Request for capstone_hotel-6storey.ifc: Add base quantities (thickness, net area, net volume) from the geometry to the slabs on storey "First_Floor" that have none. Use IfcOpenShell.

First a look at what the model holds.

```python
import ifcopenshell
import ifcopenshell.util.element
import ifcopenshell.util.unit

model = ifcopenshell.open("capstone_hotel-6storey.ifc")
print(model.schema)
for unit_type in ("LENGTHUNIT", "AREAUNIT", "VOLUMEUNIT"):
    print(unit_type, ifcopenshell.util.unit.calculate_unit_scale(model, unit_type))
storey = next(s for s in model.by_type("IfcBuildingStorey") if s.Name == "First_Floor")
slabs = [e for e in ifcopenshell.util.element.get_decomposition(storey) if e.is_a("IfcSlab")]
for e in sorted(slabs, key=lambda e: e.id()):
    print(e.id(), e.is_a(), e.Name, list(ifcopenshell.util.element.get_psets(e, qtos_only=True)), sep=" | ")
```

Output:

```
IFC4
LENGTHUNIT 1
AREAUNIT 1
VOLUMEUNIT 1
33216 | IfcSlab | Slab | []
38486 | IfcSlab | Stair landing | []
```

```python
import ifcopenshell
import ifcopenshell.api.pset
import ifcopenshell.geom
import ifcopenshell.util.element
import ifcopenshell.util.shape
import ifcopenshell.util.unit

model = ifcopenshell.open("capstone_hotel-6storey.ifc")
unit_scale = ifcopenshell.util.unit.calculate_unit_scale(model)
area_scale = ifcopenshell.util.unit.calculate_unit_scale(model, "AREAUNIT")
volume_scale = ifcopenshell.util.unit.calculate_unit_scale(model, "VOLUMEUNIT")
settings = ifcopenshell.geom.settings()

storey = next(s for s in model.by_type("IfcBuildingStorey") if s.Name == "First_Floor")
slabs = [e for e in ifcopenshell.util.element.get_decomposition(storey) if e.is_a("IfcSlab")]

for e in sorted(slabs, key=lambda e: e.id()):
    if ifcopenshell.util.element.get_psets(e, qtos_only=True, should_inherit=False):
        continue
    # Geometry comes back in metres, in the element's own axes.
    shape = ifcopenshell.geom.create_shape(settings, e)
    values = {
        "Width": ifcopenshell.util.shape.get_z(shape.geometry) / unit_scale,
        "NetArea": ifcopenshell.util.shape.get_footprint_area(shape.geometry) / area_scale,
        "NetVolume": ifcopenshell.util.shape.get_volume(shape.geometry) / volume_scale,
    }
    qto = ifcopenshell.api.pset.add_qto(model, product=e, name="Qto_SlabBaseQuantities")
    ifcopenshell.api.pset.edit_qto(model, qto=qto, properties=values)
    print(e.id(), {k: round(v, 3) for k, v in values.items()})

model.write("capstone_hotel-6storey-out.ifc")
```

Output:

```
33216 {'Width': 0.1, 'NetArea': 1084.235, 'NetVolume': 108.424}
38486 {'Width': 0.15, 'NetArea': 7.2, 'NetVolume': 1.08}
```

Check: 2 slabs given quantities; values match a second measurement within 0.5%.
